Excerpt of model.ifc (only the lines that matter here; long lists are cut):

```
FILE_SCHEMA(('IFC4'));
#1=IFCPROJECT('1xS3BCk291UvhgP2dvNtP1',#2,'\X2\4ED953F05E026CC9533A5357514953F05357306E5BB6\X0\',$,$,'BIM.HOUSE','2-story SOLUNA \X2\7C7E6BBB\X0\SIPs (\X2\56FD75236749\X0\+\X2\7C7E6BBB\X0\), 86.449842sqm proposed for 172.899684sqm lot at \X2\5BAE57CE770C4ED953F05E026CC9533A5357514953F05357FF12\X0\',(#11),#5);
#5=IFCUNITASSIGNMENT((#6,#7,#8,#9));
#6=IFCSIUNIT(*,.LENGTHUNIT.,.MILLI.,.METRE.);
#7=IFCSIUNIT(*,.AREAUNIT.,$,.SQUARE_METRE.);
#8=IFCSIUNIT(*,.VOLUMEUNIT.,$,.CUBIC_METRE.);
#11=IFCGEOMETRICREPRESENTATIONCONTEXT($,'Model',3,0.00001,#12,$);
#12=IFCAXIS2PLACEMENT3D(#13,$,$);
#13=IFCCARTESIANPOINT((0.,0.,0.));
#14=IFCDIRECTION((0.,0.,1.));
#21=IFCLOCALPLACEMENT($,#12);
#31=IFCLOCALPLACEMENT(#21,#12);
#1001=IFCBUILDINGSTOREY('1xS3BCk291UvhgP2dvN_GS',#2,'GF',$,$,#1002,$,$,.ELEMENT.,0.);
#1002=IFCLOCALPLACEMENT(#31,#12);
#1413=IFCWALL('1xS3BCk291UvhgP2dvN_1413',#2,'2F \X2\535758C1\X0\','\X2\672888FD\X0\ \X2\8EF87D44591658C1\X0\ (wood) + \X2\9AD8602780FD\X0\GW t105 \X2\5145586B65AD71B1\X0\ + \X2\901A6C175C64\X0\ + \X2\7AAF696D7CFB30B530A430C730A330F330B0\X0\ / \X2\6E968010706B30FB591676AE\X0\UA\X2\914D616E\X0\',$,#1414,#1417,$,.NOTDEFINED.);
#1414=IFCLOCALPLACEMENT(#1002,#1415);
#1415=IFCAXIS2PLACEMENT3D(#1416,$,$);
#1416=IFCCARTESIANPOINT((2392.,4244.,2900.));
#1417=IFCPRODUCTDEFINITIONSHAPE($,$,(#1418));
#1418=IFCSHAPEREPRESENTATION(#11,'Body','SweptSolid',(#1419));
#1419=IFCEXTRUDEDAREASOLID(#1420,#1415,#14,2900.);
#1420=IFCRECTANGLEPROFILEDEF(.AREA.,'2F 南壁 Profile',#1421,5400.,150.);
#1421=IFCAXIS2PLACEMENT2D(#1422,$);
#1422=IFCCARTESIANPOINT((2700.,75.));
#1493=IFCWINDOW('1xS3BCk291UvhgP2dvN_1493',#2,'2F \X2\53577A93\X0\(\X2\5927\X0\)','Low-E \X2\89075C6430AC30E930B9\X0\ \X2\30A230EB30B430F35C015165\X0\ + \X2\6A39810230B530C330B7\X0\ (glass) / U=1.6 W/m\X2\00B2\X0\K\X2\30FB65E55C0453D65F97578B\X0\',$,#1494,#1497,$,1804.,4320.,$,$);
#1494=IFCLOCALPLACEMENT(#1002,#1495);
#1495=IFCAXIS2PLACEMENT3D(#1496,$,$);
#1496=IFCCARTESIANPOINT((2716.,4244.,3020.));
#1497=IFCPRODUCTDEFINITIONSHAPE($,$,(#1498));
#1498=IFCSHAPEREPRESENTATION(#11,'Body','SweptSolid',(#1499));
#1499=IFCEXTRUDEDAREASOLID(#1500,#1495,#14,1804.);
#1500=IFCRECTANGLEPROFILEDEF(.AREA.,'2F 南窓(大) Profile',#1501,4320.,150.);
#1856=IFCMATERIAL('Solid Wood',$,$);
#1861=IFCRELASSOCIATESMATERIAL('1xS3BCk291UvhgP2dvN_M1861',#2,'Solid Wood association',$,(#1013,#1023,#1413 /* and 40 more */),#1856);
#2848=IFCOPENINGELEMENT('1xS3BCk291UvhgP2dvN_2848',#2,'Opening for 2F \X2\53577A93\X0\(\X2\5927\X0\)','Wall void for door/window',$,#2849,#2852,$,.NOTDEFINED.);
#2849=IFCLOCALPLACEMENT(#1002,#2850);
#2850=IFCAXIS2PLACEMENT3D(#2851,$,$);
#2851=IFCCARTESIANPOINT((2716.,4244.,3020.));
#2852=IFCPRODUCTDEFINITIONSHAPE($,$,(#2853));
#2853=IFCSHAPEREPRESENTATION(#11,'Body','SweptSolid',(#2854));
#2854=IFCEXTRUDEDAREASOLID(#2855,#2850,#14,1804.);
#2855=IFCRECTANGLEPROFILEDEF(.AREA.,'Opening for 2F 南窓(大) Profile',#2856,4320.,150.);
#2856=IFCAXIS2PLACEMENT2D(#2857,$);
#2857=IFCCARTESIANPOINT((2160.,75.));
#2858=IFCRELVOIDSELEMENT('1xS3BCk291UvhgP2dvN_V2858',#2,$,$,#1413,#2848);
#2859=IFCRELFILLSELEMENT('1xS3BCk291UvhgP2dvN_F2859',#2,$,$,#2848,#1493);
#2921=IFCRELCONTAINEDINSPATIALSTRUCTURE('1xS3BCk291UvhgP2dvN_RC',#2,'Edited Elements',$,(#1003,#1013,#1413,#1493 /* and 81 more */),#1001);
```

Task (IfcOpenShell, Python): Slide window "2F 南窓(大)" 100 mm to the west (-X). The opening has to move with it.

```python
import ifcopenshell
import ifcopenshell.api.geometry
import ifcopenshell.util.placement

model = ifcopenshell.open("model.ifc")

window = model.by_guid("1xS3BCk291UvhgP2dvN_1493")
opening = window.FillsVoids[0].RelatingOpeningElement
wall = opening.VoidsElements[0].RelatingBuildingElement

wall_matrix = ifcopenshell.util.placement.get_local_placement(wall.ObjectPlacement)
shift = wall_matrix[:3, 0] * -100.0
before = ifcopenshell.util.placement.get_local_placement(window.ObjectPlacement)[:3, 3].copy()

# The window is not placed relative to its opening, so move both.
for product in (opening, window):
    matrix = ifcopenshell.util.placement.get_local_placement(product.ObjectPlacement)
    matrix[:3, 3] += shift
    ifcopenshell.api.geometry.edit_object_placement(model, product=product, matrix=matrix, is_si=False)

after = ifcopenshell.util.placement.get_local_placement(window.ObjectPlacement)[:3, 3]
print("window moved by", (after - before).round(3) + 0.0)

model.write("model_rev.ifc")
```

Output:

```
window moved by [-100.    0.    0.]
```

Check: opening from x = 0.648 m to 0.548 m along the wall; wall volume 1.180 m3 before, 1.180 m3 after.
